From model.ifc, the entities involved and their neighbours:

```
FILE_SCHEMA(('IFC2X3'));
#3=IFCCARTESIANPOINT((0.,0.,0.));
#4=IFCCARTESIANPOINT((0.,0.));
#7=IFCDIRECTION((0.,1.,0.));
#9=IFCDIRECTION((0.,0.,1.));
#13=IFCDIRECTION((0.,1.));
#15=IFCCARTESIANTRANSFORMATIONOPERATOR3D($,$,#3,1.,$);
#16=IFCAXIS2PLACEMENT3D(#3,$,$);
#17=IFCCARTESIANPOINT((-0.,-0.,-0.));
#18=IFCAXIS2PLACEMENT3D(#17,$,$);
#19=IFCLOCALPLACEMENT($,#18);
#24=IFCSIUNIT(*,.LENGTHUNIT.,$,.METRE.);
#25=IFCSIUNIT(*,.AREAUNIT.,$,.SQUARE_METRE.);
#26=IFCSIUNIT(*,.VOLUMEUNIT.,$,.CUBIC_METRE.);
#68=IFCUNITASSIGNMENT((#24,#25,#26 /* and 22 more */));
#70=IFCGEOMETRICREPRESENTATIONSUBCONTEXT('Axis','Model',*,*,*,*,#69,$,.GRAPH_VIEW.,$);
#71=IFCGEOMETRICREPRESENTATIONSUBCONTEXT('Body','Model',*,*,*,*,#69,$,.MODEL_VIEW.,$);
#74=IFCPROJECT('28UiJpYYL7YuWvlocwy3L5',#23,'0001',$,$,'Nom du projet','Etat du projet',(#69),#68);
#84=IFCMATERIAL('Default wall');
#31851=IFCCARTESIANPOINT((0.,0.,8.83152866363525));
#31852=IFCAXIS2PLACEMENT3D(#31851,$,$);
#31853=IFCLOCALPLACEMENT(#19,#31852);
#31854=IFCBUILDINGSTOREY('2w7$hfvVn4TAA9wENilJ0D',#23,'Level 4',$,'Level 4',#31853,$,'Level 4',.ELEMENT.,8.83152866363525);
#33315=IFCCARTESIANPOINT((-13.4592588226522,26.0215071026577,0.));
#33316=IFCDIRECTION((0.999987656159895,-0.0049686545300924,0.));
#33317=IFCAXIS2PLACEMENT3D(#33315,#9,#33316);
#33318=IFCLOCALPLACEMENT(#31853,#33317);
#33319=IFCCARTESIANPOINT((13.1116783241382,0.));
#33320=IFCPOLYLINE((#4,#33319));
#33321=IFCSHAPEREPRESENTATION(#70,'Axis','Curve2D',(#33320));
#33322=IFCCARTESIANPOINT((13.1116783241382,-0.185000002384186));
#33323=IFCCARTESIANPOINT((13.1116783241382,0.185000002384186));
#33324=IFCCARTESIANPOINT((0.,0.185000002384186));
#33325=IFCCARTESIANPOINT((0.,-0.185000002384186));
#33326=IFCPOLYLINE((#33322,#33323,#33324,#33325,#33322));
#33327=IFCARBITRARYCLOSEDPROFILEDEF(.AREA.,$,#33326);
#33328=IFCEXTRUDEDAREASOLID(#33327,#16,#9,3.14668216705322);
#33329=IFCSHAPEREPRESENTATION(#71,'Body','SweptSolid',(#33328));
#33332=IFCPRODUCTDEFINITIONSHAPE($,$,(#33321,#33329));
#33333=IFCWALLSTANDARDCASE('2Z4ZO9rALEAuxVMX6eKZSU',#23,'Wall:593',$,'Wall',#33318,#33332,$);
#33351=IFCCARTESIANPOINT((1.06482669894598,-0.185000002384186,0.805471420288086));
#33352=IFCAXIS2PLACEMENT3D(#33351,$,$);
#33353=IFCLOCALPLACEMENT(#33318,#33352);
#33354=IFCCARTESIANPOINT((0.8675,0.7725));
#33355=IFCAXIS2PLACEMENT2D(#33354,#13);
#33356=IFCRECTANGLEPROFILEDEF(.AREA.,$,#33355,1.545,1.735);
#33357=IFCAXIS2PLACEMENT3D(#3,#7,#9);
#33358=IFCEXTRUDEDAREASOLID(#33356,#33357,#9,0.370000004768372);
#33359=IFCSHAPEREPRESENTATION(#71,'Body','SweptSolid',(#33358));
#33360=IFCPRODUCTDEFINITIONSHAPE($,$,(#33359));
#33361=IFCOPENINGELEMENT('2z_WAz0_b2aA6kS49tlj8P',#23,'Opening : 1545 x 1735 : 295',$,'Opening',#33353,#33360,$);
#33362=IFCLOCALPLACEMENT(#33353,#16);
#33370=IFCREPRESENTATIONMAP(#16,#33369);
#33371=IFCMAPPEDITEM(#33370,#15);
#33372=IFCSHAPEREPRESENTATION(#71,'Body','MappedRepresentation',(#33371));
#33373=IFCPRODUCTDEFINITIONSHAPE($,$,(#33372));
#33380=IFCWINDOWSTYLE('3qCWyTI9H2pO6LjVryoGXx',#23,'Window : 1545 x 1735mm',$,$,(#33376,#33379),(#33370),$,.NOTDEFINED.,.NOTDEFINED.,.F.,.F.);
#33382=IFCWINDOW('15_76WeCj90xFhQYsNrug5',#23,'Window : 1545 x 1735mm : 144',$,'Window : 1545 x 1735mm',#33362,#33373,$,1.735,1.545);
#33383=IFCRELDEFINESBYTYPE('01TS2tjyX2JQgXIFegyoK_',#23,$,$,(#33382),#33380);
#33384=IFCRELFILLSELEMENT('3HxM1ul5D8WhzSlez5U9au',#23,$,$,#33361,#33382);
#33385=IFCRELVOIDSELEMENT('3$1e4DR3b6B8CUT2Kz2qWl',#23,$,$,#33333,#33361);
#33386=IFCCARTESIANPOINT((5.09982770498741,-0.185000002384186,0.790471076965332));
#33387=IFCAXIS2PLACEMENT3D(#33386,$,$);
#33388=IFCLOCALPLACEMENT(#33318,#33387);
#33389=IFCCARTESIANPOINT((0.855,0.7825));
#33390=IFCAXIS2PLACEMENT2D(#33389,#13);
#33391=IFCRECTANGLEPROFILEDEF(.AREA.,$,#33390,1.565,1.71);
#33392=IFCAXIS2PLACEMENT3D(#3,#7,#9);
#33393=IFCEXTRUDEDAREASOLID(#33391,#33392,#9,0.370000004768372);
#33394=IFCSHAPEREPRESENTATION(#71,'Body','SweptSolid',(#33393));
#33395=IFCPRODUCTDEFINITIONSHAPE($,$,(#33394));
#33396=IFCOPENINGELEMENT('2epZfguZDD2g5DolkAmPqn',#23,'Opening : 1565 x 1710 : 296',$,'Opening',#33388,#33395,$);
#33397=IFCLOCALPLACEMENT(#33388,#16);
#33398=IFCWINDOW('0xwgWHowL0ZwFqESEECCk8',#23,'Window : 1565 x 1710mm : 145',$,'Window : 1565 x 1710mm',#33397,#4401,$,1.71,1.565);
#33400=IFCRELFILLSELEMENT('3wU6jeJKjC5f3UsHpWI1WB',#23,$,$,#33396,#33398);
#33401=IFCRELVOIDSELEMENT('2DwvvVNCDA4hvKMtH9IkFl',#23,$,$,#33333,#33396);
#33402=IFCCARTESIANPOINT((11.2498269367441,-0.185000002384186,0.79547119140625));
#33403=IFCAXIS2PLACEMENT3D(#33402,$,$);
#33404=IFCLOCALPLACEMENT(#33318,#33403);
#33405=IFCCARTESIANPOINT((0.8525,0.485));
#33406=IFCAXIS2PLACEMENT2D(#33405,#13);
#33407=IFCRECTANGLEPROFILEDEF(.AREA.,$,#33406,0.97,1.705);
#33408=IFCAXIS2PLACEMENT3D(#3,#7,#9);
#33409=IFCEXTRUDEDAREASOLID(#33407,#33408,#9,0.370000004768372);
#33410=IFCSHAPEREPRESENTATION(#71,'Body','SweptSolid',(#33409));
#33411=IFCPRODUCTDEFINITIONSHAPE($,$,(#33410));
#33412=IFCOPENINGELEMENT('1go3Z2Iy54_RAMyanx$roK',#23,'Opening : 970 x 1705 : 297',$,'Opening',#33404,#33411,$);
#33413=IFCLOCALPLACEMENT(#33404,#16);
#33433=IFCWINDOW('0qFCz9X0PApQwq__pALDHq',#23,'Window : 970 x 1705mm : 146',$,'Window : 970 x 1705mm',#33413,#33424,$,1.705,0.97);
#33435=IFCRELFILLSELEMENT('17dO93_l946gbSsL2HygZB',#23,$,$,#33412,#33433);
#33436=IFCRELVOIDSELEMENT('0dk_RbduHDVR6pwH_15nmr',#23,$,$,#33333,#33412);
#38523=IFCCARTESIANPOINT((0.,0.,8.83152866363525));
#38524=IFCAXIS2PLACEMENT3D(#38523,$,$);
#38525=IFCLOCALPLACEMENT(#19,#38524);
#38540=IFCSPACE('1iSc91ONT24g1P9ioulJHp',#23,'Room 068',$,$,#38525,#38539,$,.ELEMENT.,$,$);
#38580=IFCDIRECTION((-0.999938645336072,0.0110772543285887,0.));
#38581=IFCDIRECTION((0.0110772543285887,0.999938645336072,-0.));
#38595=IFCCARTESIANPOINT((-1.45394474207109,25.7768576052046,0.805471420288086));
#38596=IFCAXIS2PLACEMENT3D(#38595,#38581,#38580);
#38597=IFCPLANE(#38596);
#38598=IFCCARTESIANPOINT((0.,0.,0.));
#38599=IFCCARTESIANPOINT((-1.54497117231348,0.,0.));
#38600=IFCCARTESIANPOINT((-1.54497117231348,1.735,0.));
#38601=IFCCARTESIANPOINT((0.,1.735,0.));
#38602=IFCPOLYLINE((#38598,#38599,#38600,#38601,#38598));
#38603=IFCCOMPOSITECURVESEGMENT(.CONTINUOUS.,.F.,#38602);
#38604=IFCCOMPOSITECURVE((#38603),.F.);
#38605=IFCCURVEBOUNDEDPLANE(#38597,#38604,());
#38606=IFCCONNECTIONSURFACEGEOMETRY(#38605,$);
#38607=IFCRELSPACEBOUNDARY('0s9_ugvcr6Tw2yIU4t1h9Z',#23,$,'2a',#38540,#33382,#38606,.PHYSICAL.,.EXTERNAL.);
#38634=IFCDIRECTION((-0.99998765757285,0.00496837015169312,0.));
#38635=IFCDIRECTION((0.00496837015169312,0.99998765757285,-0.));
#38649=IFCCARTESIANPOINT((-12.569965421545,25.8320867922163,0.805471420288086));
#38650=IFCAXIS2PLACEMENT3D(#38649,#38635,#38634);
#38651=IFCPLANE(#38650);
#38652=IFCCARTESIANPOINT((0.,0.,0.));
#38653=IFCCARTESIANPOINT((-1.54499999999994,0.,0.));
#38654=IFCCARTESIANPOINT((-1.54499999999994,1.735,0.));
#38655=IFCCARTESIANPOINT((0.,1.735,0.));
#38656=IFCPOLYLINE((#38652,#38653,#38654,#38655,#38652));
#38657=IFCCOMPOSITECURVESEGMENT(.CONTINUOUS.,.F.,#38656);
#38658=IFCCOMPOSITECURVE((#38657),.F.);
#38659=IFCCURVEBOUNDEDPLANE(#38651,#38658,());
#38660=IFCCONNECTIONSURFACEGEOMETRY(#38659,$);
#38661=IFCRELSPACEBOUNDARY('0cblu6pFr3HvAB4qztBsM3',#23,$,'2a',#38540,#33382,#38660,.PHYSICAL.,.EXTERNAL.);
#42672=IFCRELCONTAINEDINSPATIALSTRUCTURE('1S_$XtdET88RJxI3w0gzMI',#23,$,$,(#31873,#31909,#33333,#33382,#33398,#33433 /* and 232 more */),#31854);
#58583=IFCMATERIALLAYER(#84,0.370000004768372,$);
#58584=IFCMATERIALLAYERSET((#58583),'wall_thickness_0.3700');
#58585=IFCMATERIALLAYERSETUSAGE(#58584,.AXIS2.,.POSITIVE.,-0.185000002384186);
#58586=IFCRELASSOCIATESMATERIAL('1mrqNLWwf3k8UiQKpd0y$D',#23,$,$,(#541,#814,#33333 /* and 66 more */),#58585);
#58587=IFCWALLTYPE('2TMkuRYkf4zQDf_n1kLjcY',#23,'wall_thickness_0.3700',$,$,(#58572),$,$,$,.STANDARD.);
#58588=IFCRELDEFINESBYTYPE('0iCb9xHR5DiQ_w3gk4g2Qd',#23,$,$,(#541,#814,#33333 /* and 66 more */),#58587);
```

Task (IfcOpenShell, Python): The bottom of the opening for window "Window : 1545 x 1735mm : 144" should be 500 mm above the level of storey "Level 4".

```python
import numpy as np
import ifcopenshell
import ifcopenshell.api.geometry
import ifcopenshell.geom
import ifcopenshell.util.element
import ifcopenshell.util.placement
import ifcopenshell.util.shape
import ifcopenshell.util.unit

model = ifcopenshell.open("model.ifc")
unit_scale = ifcopenshell.util.unit.calculate_unit_scale(model)

window = model.by_id(33382)
opening = window.FillsVoids[0].RelatingOpeningElement
storey = ifcopenshell.util.element.get_container(window, ifc_class="IfcBuildingStorey")
level = ifcopenshell.util.placement.get_local_placement(storey.ObjectPlacement)[2, 3]

# The opening's origin need not be at the sill, so measure its lowest point.
shape = ifcopenshell.geom.create_shape(ifcopenshell.geom.settings(), opening)
bottom = ifcopenshell.util.shape.get_shape_bottom_elevation(shape, shape.geometry) / unit_scale
dz = level + 0.5 / unit_scale - bottom

shift = np.array([0.0, 0.0, dz])
# The window is placed relative to its opening, so it follows when the opening moves.
matrix = ifcopenshell.util.placement.get_local_placement(opening.ObjectPlacement)
matrix[:3, 3] += shift
ifcopenshell.api.geometry.edit_object_placement(
    model, product=opening, matrix=matrix, is_si=False, should_transform_children=True
)

# Space boundary surfaces are stored in each space's coordinates; move them too.
for rel in window.ProvidesBoundaries:
    if not rel.ConnectionGeometry:
        continue
    surface = rel.ConnectionGeometry.SurfaceOnRelatingElement.BasisSurface
    space_matrix = ifcopenshell.util.placement.get_local_placement(rel.RelatingSpace.ObjectPlacement)
    point = np.array(surface.Position.Location.Coordinates) + space_matrix[:3, :3].T @ shift
    surface.Position = model.createIfcAxis2Placement3D(
        model.createIfcCartesianPoint(point.tolist()), surface.Position.Axis, surface.Position.RefDirection
    )

print(f"moved by {dz * unit_scale:+.3f} m")

model.write("model_updated.ifc")
```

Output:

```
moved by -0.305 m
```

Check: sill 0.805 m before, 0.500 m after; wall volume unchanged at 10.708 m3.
